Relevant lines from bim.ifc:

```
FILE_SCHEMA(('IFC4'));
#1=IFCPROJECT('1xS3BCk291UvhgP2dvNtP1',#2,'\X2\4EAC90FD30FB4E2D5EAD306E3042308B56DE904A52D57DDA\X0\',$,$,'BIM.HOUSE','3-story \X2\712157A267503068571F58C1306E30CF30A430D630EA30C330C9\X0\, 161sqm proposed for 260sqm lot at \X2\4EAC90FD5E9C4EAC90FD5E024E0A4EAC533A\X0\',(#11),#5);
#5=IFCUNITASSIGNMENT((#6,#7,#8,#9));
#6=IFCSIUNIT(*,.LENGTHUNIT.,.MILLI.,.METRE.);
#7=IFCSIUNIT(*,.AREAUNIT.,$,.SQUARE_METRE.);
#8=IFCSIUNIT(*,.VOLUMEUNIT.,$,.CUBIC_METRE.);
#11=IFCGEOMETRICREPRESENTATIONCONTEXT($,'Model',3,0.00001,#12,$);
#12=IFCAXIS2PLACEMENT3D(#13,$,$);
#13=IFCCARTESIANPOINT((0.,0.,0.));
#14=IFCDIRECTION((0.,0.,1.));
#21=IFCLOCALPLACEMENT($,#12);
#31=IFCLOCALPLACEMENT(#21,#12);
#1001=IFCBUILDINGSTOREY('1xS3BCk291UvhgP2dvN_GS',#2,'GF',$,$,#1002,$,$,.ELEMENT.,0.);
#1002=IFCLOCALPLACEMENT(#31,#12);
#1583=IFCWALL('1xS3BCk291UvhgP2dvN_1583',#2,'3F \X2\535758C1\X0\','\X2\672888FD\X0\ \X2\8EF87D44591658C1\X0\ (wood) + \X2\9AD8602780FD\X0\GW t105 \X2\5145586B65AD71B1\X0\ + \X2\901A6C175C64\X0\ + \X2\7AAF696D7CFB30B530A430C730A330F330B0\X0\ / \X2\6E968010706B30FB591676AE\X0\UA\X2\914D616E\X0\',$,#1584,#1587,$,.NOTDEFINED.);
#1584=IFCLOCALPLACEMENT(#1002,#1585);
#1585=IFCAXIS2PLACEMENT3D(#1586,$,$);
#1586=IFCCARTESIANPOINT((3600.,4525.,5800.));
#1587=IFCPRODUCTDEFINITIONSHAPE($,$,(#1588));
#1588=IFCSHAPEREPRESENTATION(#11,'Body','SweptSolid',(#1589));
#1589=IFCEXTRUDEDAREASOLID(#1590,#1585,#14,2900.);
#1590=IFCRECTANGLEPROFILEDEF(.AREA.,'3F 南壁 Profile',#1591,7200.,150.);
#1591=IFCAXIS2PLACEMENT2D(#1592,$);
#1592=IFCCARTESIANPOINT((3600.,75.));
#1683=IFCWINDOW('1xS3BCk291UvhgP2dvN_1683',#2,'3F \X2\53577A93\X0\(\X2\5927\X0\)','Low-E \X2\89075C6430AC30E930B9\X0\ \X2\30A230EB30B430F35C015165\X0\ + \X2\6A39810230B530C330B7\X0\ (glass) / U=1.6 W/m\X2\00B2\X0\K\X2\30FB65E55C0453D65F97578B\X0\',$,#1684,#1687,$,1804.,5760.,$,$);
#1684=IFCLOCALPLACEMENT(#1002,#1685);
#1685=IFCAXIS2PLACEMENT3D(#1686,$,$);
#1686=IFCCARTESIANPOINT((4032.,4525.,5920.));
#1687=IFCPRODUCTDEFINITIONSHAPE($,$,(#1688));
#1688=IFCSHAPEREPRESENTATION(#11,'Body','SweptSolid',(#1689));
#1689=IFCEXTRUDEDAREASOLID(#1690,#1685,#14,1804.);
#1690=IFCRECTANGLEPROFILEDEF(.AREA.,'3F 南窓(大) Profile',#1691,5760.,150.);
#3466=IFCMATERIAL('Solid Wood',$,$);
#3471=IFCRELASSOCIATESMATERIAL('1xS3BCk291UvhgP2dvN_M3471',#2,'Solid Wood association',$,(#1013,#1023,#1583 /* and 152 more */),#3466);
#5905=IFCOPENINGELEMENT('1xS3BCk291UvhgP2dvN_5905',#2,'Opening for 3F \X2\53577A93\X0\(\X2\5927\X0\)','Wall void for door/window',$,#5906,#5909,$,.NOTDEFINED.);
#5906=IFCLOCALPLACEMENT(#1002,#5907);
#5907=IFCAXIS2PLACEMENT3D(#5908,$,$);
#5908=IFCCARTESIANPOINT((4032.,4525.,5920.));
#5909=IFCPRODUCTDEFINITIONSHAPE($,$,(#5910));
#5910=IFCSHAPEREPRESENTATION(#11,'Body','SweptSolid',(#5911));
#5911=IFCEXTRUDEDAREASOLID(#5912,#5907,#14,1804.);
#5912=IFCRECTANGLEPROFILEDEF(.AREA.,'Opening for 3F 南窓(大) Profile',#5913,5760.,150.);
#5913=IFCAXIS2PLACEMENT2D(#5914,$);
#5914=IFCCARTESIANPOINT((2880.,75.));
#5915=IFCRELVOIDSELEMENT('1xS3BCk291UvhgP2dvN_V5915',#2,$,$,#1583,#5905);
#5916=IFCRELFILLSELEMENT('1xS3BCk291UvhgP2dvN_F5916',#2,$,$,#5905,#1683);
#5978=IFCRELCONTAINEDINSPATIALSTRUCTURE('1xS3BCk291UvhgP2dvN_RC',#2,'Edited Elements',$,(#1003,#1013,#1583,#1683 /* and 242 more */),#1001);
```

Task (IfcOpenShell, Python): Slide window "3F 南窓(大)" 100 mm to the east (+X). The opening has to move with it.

```python
import ifcopenshell
import ifcopenshell.api.geometry
import ifcopenshell.util.placement
import ifcopenshell.util.unit

model = ifcopenshell.open("bim.ifc")
unit_scale = ifcopenshell.util.unit.calculate_unit_scale(model)

window = model.by_guid("1xS3BCk291UvhgP2dvN_1683")
opening = window.FillsVoids[0].RelatingOpeningElement
wall = opening.VoidsElements[0].RelatingBuildingElement

wall_matrix = ifcopenshell.util.placement.get_local_placement(wall.ObjectPlacement)
shift = wall_matrix[:3, 0] * 0.1 / unit_scale
before = ifcopenshell.util.placement.get_local_placement(window.ObjectPlacement)[:3, 3].copy()

# The window is not placed relative to its opening, so move both.
for product in (opening, window):
    matrix = ifcopenshell.util.placement.get_local_placement(product.ObjectPlacement)
    matrix[:3, 3] += shift
    ifcopenshell.api.geometry.edit_object_placement(model, product=product, matrix=matrix, is_si=False)

after = ifcopenshell.util.placement.get_local_placement(window.ObjectPlacement)[:3, 3]
print("window moved by", (after - before).round(3) + 0.0)

model.write("bim_edited.ifc")
```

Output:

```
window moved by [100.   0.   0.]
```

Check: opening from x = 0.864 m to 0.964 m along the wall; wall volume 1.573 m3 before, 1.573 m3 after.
